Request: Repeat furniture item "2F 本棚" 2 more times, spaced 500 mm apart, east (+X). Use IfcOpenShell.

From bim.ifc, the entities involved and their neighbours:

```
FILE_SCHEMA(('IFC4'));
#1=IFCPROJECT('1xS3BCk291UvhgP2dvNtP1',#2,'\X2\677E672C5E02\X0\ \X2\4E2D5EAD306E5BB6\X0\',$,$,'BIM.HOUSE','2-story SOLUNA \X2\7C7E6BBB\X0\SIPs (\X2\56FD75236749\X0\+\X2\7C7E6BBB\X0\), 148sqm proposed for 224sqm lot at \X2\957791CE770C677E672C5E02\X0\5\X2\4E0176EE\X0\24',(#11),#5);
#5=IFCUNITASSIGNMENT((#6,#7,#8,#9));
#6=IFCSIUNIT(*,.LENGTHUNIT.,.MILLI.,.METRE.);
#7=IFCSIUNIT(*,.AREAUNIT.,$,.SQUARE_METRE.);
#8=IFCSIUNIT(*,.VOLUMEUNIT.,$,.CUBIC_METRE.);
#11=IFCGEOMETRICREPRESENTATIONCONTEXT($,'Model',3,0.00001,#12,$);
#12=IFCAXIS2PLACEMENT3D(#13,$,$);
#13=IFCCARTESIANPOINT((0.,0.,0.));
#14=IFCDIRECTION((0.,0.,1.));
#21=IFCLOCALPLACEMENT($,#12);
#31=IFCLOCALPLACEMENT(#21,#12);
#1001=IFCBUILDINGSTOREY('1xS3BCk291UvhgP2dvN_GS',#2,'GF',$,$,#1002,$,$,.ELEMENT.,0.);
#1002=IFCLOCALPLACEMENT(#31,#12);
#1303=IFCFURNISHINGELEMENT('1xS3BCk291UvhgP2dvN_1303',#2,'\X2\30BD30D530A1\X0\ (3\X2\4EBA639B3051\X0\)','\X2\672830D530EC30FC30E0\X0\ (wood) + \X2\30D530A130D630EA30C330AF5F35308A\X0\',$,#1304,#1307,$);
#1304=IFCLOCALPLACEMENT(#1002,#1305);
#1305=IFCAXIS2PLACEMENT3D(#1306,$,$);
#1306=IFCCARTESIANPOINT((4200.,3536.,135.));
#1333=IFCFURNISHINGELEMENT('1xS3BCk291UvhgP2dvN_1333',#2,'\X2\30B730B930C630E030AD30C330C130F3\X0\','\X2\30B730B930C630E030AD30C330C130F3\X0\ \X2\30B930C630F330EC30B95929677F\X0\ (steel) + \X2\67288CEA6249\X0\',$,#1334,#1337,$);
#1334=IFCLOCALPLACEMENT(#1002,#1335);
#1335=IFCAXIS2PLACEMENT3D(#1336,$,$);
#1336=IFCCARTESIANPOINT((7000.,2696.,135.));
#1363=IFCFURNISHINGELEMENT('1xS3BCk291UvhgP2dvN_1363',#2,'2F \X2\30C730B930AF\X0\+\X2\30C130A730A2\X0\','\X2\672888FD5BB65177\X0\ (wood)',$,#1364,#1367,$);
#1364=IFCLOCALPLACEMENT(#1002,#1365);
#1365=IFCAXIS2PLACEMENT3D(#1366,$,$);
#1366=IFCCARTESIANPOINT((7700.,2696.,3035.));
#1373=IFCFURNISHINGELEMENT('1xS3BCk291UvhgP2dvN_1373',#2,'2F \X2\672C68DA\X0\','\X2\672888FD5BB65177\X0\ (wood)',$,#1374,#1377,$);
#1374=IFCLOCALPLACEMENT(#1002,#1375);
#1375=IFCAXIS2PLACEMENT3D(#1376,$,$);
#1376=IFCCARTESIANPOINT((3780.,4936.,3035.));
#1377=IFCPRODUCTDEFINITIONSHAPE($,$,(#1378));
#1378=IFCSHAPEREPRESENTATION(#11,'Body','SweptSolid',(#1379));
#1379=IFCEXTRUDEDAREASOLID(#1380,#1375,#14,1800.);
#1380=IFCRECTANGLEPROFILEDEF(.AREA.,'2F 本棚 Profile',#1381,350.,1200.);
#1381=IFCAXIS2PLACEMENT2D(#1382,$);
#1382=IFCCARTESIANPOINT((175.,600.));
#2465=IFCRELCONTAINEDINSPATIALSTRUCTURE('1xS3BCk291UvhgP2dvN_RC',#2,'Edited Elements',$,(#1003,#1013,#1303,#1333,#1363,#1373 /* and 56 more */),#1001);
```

```python
import numpy as np
import ifcopenshell
import ifcopenshell.api.geometry
import ifcopenshell.api.root
import ifcopenshell.util.element
import ifcopenshell.util.placement

model = ifcopenshell.open("bim.ifc")


def reuse_history(source, copy):
    """copy_class also copies each property set's owner history, people and application; keep the originals."""
    for rel in copy.IsDefinedBy:
        if rel.is_a("IfcRelDefinesByProperties") and (history := rel.RelatingPropertyDefinition.OwnerHistory):
            rel.RelatingPropertyDefinition.OwnerHistory = source.OwnerHistory
            ifcopenshell.util.element.remove_deep2(model, history)


source = model.by_guid("1xS3BCk291UvhgP2dvN_1373")
base = ifcopenshell.util.placement.get_local_placement(source.ObjectPlacement)
step = np.array([1.0, 0.0, 0.0]) * 500.0

for i in range(1, 3):
    copy = ifcopenshell.api.root.copy_class(model, product=source)
    copy.Representation = ifcopenshell.util.element.copy_deep(
        model, source.Representation, exclude=["IfcGeometricRepresentationContext", "IfcRepresentationMap"]
    )
    reuse_history(source, copy)
    matrix = base.copy()
    matrix[:3, 3] += i * step
    print("added at", matrix[:3, 3].round(3) + 0.0)
    ifcopenshell.api.geometry.edit_object_placement(model, product=copy, matrix=matrix, is_si=False)

model.write("bim_updated.ifc")
```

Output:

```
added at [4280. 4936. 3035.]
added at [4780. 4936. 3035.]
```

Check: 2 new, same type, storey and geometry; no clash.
